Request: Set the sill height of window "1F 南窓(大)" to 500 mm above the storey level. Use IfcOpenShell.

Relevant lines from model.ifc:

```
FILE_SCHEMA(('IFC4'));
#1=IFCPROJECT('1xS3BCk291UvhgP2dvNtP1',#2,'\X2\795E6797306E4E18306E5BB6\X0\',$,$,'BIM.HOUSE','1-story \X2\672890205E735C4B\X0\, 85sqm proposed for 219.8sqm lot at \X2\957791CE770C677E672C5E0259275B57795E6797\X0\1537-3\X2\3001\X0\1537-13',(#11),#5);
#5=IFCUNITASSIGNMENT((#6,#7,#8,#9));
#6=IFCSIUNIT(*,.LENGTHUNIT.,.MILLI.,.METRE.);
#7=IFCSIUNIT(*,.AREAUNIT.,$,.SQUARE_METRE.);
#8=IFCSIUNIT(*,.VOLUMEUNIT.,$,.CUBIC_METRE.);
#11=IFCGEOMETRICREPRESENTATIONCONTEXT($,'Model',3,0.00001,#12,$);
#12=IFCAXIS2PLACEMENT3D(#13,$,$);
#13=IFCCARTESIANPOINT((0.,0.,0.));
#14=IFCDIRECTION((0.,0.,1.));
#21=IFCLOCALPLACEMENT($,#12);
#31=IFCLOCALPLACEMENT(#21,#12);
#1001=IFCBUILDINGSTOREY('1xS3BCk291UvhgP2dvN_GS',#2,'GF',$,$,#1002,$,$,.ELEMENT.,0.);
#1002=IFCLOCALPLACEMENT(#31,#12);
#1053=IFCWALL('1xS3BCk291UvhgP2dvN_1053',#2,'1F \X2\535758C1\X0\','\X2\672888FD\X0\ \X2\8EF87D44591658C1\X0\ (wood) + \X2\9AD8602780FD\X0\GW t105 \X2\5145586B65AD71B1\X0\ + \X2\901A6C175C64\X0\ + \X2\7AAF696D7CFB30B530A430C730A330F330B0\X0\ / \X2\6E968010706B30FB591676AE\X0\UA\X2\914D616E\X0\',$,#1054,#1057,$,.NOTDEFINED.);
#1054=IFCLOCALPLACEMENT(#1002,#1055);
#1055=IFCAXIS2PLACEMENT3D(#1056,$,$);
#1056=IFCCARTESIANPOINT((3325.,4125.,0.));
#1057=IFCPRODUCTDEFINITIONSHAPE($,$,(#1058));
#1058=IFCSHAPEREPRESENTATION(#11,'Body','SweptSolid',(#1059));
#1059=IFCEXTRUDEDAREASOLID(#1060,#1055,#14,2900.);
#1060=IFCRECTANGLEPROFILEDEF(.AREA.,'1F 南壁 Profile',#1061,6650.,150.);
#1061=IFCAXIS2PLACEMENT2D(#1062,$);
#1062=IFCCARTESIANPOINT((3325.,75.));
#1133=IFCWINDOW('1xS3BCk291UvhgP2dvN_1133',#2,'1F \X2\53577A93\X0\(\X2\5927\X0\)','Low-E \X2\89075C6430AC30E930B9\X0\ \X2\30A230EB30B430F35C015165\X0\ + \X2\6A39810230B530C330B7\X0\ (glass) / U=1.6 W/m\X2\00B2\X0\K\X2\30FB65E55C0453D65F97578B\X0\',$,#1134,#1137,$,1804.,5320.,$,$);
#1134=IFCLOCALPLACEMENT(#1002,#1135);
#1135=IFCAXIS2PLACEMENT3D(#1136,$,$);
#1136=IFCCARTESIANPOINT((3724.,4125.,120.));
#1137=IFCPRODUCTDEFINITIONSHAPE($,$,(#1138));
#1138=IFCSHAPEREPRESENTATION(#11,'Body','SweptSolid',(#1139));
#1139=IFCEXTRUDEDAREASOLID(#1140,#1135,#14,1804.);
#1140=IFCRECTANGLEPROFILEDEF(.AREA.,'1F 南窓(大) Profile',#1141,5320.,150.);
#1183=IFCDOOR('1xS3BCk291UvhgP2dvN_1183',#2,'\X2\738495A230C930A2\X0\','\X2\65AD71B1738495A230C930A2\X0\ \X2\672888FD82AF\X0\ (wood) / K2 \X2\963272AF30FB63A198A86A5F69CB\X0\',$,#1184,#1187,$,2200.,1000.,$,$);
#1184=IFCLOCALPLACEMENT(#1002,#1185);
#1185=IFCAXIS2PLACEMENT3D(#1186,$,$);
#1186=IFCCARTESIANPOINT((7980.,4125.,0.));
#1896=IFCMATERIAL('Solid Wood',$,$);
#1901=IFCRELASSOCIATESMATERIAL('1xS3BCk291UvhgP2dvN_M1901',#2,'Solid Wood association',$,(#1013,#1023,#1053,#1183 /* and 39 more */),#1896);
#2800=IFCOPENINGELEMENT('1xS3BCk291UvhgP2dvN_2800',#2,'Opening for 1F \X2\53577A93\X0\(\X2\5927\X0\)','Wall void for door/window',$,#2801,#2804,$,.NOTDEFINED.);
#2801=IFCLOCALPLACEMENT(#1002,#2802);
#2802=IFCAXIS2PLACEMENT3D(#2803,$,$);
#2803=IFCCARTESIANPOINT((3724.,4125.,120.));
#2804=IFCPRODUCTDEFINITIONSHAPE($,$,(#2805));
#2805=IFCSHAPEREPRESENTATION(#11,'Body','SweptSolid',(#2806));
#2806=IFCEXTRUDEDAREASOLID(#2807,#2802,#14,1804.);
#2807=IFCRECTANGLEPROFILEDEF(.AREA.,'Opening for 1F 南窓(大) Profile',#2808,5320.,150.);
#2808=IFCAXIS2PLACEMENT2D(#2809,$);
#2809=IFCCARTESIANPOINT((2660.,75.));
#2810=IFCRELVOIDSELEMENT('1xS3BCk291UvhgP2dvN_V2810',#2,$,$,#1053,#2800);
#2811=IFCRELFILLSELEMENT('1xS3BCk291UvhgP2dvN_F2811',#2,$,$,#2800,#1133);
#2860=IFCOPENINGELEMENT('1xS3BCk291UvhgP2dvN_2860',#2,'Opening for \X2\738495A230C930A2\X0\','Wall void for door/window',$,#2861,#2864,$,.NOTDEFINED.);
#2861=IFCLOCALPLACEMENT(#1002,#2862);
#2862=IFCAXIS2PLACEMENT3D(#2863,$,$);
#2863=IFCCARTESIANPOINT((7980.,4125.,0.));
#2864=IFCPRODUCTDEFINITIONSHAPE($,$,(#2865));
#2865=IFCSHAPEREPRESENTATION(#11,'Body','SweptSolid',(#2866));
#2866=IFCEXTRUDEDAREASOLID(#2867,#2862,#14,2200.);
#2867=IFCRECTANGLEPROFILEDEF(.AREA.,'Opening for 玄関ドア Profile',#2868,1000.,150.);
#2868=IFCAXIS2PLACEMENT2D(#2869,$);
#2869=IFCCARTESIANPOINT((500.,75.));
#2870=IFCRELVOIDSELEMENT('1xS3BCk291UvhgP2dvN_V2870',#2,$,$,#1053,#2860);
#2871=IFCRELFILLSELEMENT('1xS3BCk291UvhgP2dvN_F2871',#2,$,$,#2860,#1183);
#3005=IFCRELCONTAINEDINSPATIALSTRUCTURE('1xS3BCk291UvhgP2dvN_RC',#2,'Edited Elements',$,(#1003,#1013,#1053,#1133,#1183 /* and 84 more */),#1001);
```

```python
import numpy as np
import ifcopenshell
import ifcopenshell.api.geometry
import ifcopenshell.geom
import ifcopenshell.util.element
import ifcopenshell.util.placement
import ifcopenshell.util.shape
import ifcopenshell.util.unit

model = ifcopenshell.open("model.ifc")
unit_scale = ifcopenshell.util.unit.calculate_unit_scale(model)

window = model.by_guid("1xS3BCk291UvhgP2dvN_1133")
opening = window.FillsVoids[0].RelatingOpeningElement
storey = ifcopenshell.util.element.get_container(window, ifc_class="IfcBuildingStorey")
level = ifcopenshell.util.placement.get_local_placement(storey.ObjectPlacement)[2, 3]

# The opening's origin need not be at the sill, so measure its lowest point.
shape = ifcopenshell.geom.create_shape(ifcopenshell.geom.settings(), opening)
bottom = ifcopenshell.util.shape.get_shape_bottom_elevation(shape, shape.geometry) / unit_scale
dz = level + 500.0 - bottom

shift = np.array([0.0, 0.0, dz])
# The window is not placed relative to its opening, so move both.
for product in (opening, window):
    matrix = ifcopenshell.util.placement.get_local_placement(product.ObjectPlacement)
    matrix[:3, 3] += shift
    ifcopenshell.api.geometry.edit_object_placement(model, product=product, matrix=matrix, is_si=False)

print(f"moved by {dz * unit_scale:+.3f} m")

model.write("model-out.ifc")
```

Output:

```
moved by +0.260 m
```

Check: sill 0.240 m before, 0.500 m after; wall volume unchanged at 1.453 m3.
